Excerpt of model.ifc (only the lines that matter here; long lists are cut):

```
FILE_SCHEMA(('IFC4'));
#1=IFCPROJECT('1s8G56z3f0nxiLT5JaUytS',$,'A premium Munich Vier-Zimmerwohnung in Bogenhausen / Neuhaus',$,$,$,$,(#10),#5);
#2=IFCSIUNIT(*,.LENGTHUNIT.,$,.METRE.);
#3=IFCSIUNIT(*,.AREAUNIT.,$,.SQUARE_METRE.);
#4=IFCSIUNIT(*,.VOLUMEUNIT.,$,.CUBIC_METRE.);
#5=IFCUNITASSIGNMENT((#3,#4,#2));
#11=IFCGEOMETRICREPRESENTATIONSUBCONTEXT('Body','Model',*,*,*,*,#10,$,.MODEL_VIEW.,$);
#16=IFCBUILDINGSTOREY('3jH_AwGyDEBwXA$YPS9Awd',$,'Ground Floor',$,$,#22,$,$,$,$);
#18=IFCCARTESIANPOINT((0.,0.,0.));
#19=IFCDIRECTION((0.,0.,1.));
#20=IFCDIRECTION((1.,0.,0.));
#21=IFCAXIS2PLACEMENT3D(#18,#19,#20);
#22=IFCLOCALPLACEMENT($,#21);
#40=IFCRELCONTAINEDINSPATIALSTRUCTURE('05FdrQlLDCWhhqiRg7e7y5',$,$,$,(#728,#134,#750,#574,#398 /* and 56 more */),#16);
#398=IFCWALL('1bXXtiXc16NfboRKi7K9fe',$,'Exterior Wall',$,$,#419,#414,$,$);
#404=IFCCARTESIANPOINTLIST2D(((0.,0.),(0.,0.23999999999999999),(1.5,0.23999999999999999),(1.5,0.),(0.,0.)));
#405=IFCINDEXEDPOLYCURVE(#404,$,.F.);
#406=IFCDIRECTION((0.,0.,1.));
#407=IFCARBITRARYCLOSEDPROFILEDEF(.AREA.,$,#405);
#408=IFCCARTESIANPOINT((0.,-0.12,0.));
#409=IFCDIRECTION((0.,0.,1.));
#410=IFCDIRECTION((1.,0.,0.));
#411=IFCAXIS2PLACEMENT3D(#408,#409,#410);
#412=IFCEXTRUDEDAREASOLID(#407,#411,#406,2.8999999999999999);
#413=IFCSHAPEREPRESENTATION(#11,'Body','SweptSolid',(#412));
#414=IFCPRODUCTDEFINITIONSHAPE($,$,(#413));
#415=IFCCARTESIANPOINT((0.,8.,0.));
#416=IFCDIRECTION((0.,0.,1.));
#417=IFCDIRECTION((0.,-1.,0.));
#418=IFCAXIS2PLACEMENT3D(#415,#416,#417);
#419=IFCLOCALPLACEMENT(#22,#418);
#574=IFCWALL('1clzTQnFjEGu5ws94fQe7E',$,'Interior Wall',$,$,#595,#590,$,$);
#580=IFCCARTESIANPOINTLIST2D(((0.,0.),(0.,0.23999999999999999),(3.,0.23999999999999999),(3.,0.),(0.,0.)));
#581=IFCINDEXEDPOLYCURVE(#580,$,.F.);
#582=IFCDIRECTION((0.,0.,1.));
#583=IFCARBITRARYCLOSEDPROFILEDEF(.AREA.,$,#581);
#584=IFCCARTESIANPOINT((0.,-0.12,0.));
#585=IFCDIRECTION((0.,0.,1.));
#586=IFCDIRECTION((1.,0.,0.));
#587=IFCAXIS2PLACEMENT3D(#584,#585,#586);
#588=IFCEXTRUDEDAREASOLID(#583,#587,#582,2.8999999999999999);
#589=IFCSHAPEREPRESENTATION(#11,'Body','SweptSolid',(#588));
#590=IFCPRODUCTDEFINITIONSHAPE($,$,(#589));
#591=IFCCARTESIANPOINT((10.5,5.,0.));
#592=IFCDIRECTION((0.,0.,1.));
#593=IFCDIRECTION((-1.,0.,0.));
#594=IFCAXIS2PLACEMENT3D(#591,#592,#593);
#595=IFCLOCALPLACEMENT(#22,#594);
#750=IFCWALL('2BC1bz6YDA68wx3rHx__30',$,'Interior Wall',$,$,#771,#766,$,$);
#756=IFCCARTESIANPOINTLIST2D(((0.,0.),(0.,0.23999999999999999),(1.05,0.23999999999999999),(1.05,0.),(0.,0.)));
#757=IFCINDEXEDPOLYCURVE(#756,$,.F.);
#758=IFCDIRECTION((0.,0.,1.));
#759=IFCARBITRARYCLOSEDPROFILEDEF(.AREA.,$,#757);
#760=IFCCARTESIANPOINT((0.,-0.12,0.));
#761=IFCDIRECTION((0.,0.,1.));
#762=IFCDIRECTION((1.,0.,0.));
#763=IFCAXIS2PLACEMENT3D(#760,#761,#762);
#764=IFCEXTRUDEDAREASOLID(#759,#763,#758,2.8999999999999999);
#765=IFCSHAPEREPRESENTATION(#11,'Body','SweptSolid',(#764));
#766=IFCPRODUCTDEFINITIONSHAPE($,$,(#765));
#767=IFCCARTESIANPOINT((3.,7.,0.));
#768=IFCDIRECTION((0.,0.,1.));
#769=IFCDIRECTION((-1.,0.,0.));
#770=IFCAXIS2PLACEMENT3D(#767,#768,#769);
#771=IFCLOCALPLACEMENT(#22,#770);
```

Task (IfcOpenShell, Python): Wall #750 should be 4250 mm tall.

```python
import ifcopenshell
import ifcopenshell.geom
import ifcopenshell.util.representation
import ifcopenshell.util.shape

model = ifcopenshell.open("model.ifc")
settings = ifcopenshell.geom.settings()


def volume(element):
    """Net volume in cubic metres, openings subtracted."""
    shape = ifcopenshell.geom.create_shape(settings, element)
    return ifcopenshell.util.shape.get_volume(shape.geometry)


wall = model.by_guid("2BC1bz6YDA68wx3rHx__30")
before = volume(wall)

body = ifcopenshell.util.representation.get_representation(wall, "Model", "Body")
solid = body.Items[0]
old_height = solid.Depth
solid.Depth = 4.25
after = volume(wall)

print(f"height {old_height:g} -> {solid.Depth:g}, volume {before:.3f} -> {after:.3f} m3")

model.write("model_edited.ifc")
```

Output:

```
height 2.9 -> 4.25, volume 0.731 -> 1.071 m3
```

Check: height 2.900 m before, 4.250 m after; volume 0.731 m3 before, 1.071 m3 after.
